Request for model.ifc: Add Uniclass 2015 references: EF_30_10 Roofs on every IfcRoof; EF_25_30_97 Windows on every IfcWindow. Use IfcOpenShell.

First a look at what the model holds.

```python
import ifcopenshell

model = ifcopenshell.open("model.ifc")
print(model.schema)
print("classifications:", [c.Name for c in model.by_type("IfcClassification")])
for ifc_class in ("IfcDoor", "IfcRoof", "IfcStair", "IfcWall", "IfcWindow"):
    print(ifc_class, len(model.by_type(ifc_class)))
```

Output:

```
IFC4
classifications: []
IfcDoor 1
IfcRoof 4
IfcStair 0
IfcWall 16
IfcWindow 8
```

```python
import ifcopenshell
import ifcopenshell.api.classification

model = ifcopenshell.open("model.ifc")

system = ifcopenshell.api.classification.add_classification(model, classification="Uniclass 2015")

codes = {
    "IfcRoof": ("EF_30_10", "Roofs"),
    "IfcWindow": ("EF_25_30_97", "Windows"),
}
for ifc_class, (code, name) in codes.items():
    products = model.by_type(ifc_class)
    ifcopenshell.api.classification.add_reference(
        model, products=products, classification=system, identification=code, name=name
    )
    print(code, len(products))

model.write("model_v2.ifc")
```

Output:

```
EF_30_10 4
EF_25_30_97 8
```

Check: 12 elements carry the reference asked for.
